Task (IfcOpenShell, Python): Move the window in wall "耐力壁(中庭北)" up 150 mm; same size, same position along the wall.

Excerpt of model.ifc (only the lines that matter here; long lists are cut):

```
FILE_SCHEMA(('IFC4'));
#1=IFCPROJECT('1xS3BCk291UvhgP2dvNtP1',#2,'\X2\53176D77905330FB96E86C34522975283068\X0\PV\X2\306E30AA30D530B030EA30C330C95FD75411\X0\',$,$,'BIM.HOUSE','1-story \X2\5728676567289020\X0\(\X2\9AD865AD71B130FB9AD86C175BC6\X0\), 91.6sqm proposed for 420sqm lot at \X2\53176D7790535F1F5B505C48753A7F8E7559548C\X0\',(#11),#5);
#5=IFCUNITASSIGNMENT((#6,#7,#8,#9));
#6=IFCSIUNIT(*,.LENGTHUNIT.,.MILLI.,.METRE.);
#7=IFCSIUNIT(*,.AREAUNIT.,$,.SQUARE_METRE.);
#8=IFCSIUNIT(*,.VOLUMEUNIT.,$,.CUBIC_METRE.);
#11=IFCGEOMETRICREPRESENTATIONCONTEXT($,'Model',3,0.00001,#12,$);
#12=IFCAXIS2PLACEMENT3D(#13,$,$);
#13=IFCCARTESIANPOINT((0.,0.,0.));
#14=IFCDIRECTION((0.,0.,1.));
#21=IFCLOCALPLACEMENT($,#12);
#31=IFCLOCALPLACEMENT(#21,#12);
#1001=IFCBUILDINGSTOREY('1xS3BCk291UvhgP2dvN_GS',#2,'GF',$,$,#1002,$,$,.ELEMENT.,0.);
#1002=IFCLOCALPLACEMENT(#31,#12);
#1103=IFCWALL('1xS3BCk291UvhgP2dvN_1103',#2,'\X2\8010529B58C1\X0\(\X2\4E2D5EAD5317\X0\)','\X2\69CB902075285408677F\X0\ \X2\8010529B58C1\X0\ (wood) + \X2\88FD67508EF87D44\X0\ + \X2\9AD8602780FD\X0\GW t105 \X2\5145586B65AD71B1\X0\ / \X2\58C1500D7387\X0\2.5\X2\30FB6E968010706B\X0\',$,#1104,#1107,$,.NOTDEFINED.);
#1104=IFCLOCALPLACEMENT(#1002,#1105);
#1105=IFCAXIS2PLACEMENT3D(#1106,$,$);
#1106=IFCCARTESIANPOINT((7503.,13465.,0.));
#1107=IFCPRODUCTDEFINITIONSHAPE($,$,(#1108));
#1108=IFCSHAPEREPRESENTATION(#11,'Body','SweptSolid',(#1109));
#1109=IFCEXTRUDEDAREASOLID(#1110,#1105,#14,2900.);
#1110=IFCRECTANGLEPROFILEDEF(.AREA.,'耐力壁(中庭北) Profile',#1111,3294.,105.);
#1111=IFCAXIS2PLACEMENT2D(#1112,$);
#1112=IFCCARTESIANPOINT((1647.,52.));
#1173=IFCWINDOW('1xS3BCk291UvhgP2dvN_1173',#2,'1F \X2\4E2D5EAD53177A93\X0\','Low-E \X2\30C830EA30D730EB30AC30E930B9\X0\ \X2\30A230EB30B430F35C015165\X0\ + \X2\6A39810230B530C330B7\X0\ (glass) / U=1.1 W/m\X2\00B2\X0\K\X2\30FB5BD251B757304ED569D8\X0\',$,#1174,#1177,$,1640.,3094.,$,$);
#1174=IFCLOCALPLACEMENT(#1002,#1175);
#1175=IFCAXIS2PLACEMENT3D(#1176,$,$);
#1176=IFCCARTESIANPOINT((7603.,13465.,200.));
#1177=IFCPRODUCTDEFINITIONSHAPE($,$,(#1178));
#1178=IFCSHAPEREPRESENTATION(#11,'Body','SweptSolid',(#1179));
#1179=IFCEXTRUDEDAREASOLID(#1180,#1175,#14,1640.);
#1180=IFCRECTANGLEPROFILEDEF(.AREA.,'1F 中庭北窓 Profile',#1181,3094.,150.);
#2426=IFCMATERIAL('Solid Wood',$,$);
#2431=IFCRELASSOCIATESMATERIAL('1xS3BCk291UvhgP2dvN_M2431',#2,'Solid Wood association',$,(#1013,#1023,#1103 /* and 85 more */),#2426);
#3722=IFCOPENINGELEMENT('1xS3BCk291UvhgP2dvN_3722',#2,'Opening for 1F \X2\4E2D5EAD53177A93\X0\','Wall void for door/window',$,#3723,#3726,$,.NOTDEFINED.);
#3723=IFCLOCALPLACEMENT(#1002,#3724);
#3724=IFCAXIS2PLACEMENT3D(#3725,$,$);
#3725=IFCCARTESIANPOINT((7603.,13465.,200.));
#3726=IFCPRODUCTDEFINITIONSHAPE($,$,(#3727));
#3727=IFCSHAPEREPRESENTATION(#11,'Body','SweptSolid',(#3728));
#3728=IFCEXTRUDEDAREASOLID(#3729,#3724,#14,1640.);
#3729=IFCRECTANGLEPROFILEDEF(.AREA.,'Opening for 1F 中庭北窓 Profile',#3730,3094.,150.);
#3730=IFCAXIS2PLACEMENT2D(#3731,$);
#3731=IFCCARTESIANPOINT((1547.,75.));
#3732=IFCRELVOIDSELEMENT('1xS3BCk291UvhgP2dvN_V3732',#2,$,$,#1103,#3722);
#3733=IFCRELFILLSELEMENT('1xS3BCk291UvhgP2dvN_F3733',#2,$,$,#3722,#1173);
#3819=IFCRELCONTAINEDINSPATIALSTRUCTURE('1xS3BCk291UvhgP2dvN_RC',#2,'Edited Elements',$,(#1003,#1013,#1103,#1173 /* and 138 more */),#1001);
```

```python
import numpy as np
import ifcopenshell
import ifcopenshell.api.geometry
import ifcopenshell.util.placement
import ifcopenshell.util.unit

model = ifcopenshell.open("model.ifc")
unit_scale = ifcopenshell.util.unit.calculate_unit_scale(model)

window = model.by_guid("1xS3BCk291UvhgP2dvN_1173")
opening = window.FillsVoids[0].RelatingOpeningElement
dz = 150.0

shift = np.array([0.0, 0.0, dz])
# The window is not placed relative to its opening, so move both.
for product in (opening, window):
    matrix = ifcopenshell.util.placement.get_local_placement(product.ObjectPlacement)
    matrix[:3, 3] += shift
    ifcopenshell.api.geometry.edit_object_placement(model, product=product, matrix=matrix, is_si=False)

print(f"moved by {dz * unit_scale:+.3f} m")

model.write("model_v2.ifc")
```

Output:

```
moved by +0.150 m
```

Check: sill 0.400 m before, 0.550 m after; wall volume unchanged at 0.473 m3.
